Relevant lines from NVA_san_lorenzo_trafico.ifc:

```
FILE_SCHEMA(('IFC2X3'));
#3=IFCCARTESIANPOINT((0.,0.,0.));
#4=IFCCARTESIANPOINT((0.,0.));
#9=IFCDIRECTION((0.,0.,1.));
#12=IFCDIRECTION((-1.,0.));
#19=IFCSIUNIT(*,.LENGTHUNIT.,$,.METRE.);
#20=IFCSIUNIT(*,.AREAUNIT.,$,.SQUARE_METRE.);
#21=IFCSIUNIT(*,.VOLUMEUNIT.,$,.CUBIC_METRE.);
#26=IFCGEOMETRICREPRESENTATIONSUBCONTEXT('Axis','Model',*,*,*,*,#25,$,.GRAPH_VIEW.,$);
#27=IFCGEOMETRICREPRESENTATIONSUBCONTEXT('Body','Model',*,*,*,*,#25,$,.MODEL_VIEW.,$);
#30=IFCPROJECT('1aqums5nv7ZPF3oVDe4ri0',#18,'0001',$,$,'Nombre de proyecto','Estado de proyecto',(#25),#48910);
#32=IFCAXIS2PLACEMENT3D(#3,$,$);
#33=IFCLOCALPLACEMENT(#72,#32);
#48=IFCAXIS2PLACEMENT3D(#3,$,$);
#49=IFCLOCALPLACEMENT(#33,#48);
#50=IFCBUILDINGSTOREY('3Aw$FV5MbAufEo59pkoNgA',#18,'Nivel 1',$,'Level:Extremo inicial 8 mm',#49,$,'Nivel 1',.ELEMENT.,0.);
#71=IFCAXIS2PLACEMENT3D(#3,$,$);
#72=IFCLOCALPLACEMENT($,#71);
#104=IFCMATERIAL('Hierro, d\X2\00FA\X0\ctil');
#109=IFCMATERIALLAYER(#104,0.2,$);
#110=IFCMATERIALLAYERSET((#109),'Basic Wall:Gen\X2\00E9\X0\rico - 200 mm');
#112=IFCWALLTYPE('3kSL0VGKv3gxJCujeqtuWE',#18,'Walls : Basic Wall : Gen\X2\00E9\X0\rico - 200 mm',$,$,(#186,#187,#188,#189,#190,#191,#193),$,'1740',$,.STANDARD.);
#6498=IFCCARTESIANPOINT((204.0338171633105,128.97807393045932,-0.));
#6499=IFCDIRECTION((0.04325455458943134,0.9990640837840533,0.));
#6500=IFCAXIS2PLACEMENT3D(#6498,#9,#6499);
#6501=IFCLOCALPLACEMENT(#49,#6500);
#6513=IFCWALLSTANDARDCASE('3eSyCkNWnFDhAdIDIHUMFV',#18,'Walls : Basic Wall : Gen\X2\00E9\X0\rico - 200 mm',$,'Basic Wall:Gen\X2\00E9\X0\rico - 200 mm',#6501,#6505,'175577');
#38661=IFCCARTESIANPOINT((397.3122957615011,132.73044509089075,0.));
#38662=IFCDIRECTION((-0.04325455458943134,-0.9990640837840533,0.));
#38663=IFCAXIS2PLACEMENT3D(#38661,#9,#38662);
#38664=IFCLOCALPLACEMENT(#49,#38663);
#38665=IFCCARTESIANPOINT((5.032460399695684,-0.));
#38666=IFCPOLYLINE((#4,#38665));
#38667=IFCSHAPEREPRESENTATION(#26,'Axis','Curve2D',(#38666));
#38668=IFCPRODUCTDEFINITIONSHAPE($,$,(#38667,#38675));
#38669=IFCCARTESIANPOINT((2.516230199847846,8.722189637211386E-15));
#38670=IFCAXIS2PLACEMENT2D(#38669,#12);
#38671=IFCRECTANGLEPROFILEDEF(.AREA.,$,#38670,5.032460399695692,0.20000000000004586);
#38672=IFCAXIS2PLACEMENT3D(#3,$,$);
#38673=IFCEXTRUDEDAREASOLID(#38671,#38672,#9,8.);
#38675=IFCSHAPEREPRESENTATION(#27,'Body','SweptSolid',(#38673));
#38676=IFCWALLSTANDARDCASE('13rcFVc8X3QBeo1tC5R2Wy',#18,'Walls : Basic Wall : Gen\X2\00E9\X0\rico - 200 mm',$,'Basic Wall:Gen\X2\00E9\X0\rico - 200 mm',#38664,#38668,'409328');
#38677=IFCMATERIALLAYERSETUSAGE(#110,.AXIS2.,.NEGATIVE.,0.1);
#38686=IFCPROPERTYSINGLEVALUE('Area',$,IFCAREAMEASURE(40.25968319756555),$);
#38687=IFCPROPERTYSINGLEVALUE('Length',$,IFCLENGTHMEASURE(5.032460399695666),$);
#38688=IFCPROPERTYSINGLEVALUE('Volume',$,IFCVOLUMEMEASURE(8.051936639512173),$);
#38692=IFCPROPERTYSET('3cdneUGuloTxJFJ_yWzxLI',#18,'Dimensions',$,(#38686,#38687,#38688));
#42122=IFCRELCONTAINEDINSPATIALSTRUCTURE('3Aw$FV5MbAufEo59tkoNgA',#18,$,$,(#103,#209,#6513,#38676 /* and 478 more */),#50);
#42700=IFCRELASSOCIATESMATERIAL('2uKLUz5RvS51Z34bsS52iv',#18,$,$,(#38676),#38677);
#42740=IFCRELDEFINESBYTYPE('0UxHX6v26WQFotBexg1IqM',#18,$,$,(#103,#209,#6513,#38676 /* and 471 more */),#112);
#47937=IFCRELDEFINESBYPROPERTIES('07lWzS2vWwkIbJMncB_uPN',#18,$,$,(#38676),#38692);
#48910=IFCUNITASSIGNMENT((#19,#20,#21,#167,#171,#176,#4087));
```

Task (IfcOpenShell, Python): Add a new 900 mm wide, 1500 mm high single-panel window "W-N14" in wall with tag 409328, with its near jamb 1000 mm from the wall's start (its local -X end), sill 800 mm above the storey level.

```python
import numpy as np
import ifcopenshell
import ifcopenshell.api.feature
import ifcopenshell.api.geometry
import ifcopenshell.api.pset
import ifcopenshell.api.root
import ifcopenshell.api.spatial
import ifcopenshell.api.type
import ifcopenshell.geom
import ifcopenshell.util.element
import ifcopenshell.util.placement
import ifcopenshell.util.representation
import ifcopenshell.util.shape
import ifcopenshell.util.unit

model = ifcopenshell.open("NVA_san_lorenzo_trafico.ifc")
unit_scale = ifcopenshell.util.unit.calculate_unit_scale(model)
area_scale = ifcopenshell.util.unit.calculate_unit_scale(model, "AREAUNIT")
volume_scale = ifcopenshell.util.unit.calculate_unit_scale(model, "VOLUMEUNIT")
settings = ifcopenshell.geom.settings()


def volume(element):
    """Net volume in cubic metres, openings subtracted."""
    shape = ifcopenshell.geom.create_shape(settings, element)
    return ifcopenshell.util.shape.get_volume(shape.geometry)


wall = model.by_guid("13rcFVc8X3QBeo1tC5R2Wy")
storey = ifcopenshell.util.element.get_container(wall, ifc_class="IfcBuildingStorey")
context = ifcopenshell.util.representation.get_context(model, "Model", "Body", "MODEL_VIEW")
before = volume(wall)

width, height, from_end, sill = 0.9, 1.5, 1, 0.8  # metres

# The wall runs along its own X axis, and the end named is its -X end.
wall_shape = ifcopenshell.geom.create_shape(settings, wall)
x, y, z = ifcopenshell.util.shape.get_vertices(wall_shape.geometry).T
start = x.min() + from_end
face, thickness = float(y.min()), float(y.max() - y.min())
wall_matrix = ifcopenshell.util.placement.get_local_placement(wall.ObjectPlacement)
level = ifcopenshell.util.placement.get_local_placement(storey.ObjectPlacement)[2, 3]


def in_wall(x, y):
    """Placement at x, y metres in the wall's axes, at sill height."""
    matrix = wall_matrix.copy()
    matrix[:, 3] = wall_matrix @ np.array([x / unit_scale, y / unit_scale, 0.0, 1.0])
    matrix[2, 3] = level + sill / unit_scale
    return matrix


# Opening: a box that overshoots both wall faces by 50 mm.
opening = ifcopenshell.api.root.create_entity(model, ifc_class="IfcOpeningElement")
box = ifcopenshell.api.geometry.add_wall_representation(
    model, context=context, length=width, height=height, thickness=thickness + 0.1
)
ifcopenshell.api.geometry.assign_representation(model, product=opening, representation=box)
ifcopenshell.api.geometry.edit_object_placement(model, product=opening, matrix=in_wall(start, face - 0.05), is_si=False)
ifcopenshell.api.feature.add_feature(model, feature=opening, element=wall)

window = ifcopenshell.api.root.create_entity(model, ifc_class="IfcWindow", name="W-N14")
window.OverallWidth, window.OverallHeight = width / unit_scale, height / unit_scale
body = ifcopenshell.api.geometry.add_window_representation(
    model,
    context=context,
    overall_width=window.OverallWidth,
    overall_height=window.OverallHeight,
    partition_type="SINGLE_PANEL",
)
ifcopenshell.api.geometry.assign_representation(model, product=window, representation=body)
ifcopenshell.api.spatial.assign_container(model, products=[window], relating_structure=storey)
fills = ifcopenshell.api.feature.add_filling(model, opening=opening, element=window)
fills.OwnerHistory = window.OwnerHistory  # required in IFC2X3

# IFC2X3 keeps the operation on the window style.
style = ifcopenshell.api.root.create_entity(model, ifc_class="IfcWindowStyle", name="W-N14")
style.OperationType, style.ConstructionType = "SINGLE_PANEL", "NOTDEFINED"
style.ParameterTakesPrecedence = style.Sizeable = False
ifcopenshell.api.type.assign_type(model, related_objects=[window], relating_type=style)

# Centre the window in the wall's thickness.
ifcopenshell.api.geometry.edit_object_placement(model, product=window, matrix=in_wall(start, face), is_si=False)
window_shape = ifcopenshell.geom.create_shape(settings, window)
depth = ifcopenshell.util.shape.get_vertices(window_shape.geometry)[:, 1]
offset = face + thickness / 2 - (depth.min() + depth.max()) / 2
ifcopenshell.api.geometry.edit_object_placement(model, product=window, matrix=in_wall(start, offset), is_si=False)

after = volume(wall)

# Update the wall's stored quantities.
pset = model.by_id(ifcopenshell.util.element.get_pset(wall, "Dimensions", should_inherit=False)["id"])
ifcopenshell.api.pset.edit_pset(model, pset=pset, properties={
    "Area": model.create_entity("IfcAreaMeasure", after / thickness / area_scale),
    "Volume": model.create_entity("IfcVolumeMeasure", after / volume_scale),
})

print(f"wall volume {before:.3f} -> {after:.3f} m3")

model.write("NVA_san_lorenzo_trafico_v2.ifc")
```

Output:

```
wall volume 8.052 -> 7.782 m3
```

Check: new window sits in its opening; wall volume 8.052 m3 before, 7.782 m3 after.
